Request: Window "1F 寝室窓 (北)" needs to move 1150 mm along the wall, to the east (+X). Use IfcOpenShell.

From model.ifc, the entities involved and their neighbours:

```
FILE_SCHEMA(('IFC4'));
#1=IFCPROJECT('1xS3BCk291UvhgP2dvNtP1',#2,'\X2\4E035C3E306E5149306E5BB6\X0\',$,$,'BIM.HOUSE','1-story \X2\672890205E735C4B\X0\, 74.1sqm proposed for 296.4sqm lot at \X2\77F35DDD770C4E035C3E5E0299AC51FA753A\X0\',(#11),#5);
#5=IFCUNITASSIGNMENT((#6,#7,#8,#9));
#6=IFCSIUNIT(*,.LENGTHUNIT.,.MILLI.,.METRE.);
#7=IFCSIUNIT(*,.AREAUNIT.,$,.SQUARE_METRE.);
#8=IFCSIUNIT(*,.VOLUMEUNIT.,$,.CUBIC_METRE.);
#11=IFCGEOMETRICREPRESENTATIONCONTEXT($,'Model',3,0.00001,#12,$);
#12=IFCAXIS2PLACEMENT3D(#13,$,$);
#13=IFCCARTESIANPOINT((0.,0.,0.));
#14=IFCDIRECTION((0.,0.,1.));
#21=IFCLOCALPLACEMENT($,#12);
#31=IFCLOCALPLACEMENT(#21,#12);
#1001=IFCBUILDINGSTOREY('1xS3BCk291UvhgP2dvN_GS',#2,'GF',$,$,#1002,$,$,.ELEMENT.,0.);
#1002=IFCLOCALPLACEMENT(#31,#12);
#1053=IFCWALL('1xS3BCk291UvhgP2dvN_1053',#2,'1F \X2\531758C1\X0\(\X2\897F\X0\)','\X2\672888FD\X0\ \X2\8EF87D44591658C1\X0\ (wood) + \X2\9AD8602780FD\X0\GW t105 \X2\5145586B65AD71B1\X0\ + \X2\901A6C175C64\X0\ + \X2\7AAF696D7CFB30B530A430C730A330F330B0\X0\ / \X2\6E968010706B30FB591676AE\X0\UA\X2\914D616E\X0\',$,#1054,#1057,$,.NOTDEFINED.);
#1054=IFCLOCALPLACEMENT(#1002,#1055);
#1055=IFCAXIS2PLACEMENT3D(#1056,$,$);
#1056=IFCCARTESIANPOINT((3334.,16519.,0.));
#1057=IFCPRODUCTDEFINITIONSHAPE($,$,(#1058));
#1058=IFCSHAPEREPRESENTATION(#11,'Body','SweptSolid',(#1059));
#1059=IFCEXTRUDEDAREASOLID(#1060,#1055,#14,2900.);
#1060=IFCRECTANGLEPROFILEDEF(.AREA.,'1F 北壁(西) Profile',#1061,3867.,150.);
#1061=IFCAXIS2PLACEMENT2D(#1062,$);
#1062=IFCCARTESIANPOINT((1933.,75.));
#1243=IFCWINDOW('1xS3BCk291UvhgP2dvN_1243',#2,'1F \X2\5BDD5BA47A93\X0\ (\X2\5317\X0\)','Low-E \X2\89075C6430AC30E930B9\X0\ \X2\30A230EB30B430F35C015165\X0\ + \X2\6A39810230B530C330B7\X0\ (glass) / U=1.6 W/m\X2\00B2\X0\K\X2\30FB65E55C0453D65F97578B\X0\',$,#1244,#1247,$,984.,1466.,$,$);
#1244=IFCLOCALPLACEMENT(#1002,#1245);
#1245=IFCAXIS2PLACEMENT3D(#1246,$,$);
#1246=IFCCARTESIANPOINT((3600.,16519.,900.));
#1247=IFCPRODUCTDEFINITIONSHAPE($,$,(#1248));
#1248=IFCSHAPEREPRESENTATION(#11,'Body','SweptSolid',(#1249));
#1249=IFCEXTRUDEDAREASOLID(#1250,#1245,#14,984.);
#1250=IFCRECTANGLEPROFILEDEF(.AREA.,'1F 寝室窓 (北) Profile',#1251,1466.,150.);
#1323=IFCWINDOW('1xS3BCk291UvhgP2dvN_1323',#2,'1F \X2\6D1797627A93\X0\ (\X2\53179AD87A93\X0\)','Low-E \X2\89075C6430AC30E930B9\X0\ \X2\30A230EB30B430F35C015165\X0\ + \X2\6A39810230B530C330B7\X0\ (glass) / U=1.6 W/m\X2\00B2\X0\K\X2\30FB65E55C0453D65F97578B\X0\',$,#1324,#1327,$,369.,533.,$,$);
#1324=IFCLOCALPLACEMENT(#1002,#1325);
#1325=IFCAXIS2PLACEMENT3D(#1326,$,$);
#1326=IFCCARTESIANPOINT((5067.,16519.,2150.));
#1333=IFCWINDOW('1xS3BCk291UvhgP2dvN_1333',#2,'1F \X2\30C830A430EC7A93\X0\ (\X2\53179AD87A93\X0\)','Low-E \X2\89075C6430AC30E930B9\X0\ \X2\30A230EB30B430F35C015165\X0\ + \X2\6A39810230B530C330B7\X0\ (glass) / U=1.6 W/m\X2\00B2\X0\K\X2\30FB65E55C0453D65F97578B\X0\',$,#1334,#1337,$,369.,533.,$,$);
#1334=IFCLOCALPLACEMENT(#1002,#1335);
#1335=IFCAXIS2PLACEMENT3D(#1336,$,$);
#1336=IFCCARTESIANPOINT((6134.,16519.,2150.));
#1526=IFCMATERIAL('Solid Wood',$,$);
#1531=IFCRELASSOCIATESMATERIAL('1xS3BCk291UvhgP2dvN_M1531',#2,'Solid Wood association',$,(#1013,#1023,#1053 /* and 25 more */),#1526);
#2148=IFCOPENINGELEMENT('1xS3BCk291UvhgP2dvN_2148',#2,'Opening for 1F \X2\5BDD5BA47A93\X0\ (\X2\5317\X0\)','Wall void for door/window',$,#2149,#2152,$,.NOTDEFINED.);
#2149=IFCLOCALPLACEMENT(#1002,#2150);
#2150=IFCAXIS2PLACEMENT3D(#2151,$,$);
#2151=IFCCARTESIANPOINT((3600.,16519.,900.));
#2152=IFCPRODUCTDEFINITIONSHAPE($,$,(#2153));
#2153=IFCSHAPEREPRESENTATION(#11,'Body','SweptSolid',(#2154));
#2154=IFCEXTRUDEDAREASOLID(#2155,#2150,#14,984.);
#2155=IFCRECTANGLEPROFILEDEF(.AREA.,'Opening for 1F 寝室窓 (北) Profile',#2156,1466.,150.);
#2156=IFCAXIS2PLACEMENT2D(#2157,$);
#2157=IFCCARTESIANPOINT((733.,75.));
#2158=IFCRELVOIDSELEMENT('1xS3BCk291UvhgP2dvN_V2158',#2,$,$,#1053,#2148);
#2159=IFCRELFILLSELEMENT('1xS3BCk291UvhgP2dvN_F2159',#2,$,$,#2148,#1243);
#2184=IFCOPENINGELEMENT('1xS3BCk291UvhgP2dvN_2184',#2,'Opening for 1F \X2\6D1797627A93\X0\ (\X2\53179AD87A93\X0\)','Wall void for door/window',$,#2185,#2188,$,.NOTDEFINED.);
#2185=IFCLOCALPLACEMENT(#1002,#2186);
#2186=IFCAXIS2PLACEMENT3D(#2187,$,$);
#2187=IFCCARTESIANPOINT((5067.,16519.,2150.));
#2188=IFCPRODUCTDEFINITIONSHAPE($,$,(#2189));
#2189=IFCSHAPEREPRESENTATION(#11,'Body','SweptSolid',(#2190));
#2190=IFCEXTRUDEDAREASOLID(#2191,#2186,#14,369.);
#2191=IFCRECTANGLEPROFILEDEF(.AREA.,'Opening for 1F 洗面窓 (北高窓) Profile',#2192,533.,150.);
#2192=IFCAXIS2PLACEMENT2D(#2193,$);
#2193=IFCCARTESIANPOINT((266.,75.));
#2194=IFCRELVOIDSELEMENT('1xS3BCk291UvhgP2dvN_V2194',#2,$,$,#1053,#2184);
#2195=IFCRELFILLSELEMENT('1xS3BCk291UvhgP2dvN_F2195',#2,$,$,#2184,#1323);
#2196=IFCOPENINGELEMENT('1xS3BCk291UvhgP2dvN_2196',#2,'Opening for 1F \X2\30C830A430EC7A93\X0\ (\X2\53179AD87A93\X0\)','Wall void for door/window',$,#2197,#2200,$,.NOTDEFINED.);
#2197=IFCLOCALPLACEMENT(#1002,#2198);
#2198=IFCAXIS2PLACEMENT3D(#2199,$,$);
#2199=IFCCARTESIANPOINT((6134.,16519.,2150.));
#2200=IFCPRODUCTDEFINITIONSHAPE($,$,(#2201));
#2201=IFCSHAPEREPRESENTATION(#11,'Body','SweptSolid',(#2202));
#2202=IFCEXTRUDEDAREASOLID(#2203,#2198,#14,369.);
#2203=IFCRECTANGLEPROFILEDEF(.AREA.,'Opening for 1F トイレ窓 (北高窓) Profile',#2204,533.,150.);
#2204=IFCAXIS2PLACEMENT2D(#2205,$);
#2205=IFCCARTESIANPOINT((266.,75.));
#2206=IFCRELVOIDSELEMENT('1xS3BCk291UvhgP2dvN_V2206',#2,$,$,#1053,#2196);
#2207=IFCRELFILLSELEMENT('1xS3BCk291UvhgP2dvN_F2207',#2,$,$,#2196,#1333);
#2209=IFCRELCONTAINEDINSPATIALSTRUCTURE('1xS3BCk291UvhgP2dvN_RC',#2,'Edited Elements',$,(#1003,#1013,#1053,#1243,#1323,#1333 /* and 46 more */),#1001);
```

```python
import ifcopenshell
import ifcopenshell.api.geometry
import ifcopenshell.util.placement
import ifcopenshell.util.unit

model = ifcopenshell.open("model.ifc")
unit_scale = ifcopenshell.util.unit.calculate_unit_scale(model)

window = model.by_guid("1xS3BCk291UvhgP2dvN_1243")
opening = window.FillsVoids[0].RelatingOpeningElement
wall = opening.VoidsElements[0].RelatingBuildingElement

wall_matrix = ifcopenshell.util.placement.get_local_placement(wall.ObjectPlacement)
shift = wall_matrix[:3, 0] * 1.15 / unit_scale
before = ifcopenshell.util.placement.get_local_placement(window.ObjectPlacement)[:3, 3].copy()

# The window is not placed relative to its opening, so move both.
for product in (opening, window):
    matrix = ifcopenshell.util.placement.get_local_placement(product.ObjectPlacement)
    matrix[:3, 3] += shift
    ifcopenshell.api.geometry.edit_object_placement(model, product=product, matrix=matrix, is_si=False)

after = ifcopenshell.util.placement.get_local_placement(window.ObjectPlacement)[:3, 3]
print("window moved by", (after - before).round(3) + 0.0)

model.write("model_edited.ifc")
```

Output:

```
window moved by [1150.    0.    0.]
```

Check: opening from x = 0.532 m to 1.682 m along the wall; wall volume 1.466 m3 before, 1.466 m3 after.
